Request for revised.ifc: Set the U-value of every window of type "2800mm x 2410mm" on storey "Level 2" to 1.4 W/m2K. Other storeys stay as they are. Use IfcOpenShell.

First a look at what the model holds.

```python
import ifcopenshell
import ifcopenshell.util.element

model = ifcopenshell.open("revised.ifc")
print(model.schema)
storey = next(s for s in model.by_type("IfcBuildingStorey") if s.Name == "Level 2")
windows = [e for e in ifcopenshell.util.element.get_decomposition(storey) if e.is_a("IfcWindow")]
seen = {}
for e in windows:
    element_type = ifcopenshell.util.element.get_type(e)
    key = (element_type.Name if element_type != e and element_type else None, ifcopenshell.util.element.get_pset(e, "Pset_WindowCommon", "ThermalTransmittance"))
    seen[key] = seen.get(key, 0) + 1
for (name, value), count in sorted(seen.items(), key=str):
    print(count, "x", name, "|", value)
```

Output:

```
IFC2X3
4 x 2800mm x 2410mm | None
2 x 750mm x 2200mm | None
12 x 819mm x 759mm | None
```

```python
import ifcopenshell
import ifcopenshell.api.pset
import ifcopenshell.util.element

model = ifcopenshell.open("revised.ifc")

storey = next(s for s in model.by_type("IfcBuildingStorey") if s.Name == "Level 2")
windows = [e for e in ifcopenshell.util.element.get_decomposition(storey) if e.is_a("IfcWindow")]

count = 0
for e in windows:
    element_type = ifcopenshell.util.element.get_type(e)
    if element_type in (None, e) or element_type.Name != "2800mm x 2410mm":
        continue
    # add_pset returns the element's existing set when there is one.
    pset = ifcopenshell.api.pset.add_pset(model, product=e, name="Pset_WindowCommon")
    ifcopenshell.api.pset.edit_pset(model, pset=pset, properties={"ThermalTransmittance": 1.4})
    count += 1

print(count, "windows updated")

model.write("revised_v2.ifc")
```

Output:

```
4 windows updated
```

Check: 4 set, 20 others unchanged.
